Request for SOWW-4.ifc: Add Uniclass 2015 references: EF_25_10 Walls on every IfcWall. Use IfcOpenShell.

First a look at what the model holds.

```python
import ifcopenshell

model = ifcopenshell.open("SOWW-4.ifc")
print(model.schema)
print("classifications:", [c.Name for c in model.by_type("IfcClassification")])
for ifc_class in ("IfcDoor", "IfcRoof", "IfcStair", "IfcWall", "IfcWindow"):
    print(ifc_class, len(model.by_type(ifc_class)))
```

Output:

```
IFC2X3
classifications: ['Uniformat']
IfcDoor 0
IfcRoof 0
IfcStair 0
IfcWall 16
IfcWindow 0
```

```python
import ifcopenshell
import ifcopenshell.api.classification

model = ifcopenshell.open("SOWW-4.ifc")

# IFC2X3 requires Source and Edition and has no link from the project to the system.
system = model.create_entity("IfcClassification", Source="NBS", Edition="2015", Name="Uniclass 2015")

codes = {
    "IfcWall": ("EF_25_10", "Walls"),
}
for ifc_class, (code, name) in codes.items():
    products = model.by_type(ifc_class)
    ifcopenshell.api.classification.add_reference(
        model, products=products, classification=system, identification=code, name=name
    )
    print(code, len(products))

model.write("SOWW-4_v2.ifc")
```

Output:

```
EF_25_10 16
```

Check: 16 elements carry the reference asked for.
